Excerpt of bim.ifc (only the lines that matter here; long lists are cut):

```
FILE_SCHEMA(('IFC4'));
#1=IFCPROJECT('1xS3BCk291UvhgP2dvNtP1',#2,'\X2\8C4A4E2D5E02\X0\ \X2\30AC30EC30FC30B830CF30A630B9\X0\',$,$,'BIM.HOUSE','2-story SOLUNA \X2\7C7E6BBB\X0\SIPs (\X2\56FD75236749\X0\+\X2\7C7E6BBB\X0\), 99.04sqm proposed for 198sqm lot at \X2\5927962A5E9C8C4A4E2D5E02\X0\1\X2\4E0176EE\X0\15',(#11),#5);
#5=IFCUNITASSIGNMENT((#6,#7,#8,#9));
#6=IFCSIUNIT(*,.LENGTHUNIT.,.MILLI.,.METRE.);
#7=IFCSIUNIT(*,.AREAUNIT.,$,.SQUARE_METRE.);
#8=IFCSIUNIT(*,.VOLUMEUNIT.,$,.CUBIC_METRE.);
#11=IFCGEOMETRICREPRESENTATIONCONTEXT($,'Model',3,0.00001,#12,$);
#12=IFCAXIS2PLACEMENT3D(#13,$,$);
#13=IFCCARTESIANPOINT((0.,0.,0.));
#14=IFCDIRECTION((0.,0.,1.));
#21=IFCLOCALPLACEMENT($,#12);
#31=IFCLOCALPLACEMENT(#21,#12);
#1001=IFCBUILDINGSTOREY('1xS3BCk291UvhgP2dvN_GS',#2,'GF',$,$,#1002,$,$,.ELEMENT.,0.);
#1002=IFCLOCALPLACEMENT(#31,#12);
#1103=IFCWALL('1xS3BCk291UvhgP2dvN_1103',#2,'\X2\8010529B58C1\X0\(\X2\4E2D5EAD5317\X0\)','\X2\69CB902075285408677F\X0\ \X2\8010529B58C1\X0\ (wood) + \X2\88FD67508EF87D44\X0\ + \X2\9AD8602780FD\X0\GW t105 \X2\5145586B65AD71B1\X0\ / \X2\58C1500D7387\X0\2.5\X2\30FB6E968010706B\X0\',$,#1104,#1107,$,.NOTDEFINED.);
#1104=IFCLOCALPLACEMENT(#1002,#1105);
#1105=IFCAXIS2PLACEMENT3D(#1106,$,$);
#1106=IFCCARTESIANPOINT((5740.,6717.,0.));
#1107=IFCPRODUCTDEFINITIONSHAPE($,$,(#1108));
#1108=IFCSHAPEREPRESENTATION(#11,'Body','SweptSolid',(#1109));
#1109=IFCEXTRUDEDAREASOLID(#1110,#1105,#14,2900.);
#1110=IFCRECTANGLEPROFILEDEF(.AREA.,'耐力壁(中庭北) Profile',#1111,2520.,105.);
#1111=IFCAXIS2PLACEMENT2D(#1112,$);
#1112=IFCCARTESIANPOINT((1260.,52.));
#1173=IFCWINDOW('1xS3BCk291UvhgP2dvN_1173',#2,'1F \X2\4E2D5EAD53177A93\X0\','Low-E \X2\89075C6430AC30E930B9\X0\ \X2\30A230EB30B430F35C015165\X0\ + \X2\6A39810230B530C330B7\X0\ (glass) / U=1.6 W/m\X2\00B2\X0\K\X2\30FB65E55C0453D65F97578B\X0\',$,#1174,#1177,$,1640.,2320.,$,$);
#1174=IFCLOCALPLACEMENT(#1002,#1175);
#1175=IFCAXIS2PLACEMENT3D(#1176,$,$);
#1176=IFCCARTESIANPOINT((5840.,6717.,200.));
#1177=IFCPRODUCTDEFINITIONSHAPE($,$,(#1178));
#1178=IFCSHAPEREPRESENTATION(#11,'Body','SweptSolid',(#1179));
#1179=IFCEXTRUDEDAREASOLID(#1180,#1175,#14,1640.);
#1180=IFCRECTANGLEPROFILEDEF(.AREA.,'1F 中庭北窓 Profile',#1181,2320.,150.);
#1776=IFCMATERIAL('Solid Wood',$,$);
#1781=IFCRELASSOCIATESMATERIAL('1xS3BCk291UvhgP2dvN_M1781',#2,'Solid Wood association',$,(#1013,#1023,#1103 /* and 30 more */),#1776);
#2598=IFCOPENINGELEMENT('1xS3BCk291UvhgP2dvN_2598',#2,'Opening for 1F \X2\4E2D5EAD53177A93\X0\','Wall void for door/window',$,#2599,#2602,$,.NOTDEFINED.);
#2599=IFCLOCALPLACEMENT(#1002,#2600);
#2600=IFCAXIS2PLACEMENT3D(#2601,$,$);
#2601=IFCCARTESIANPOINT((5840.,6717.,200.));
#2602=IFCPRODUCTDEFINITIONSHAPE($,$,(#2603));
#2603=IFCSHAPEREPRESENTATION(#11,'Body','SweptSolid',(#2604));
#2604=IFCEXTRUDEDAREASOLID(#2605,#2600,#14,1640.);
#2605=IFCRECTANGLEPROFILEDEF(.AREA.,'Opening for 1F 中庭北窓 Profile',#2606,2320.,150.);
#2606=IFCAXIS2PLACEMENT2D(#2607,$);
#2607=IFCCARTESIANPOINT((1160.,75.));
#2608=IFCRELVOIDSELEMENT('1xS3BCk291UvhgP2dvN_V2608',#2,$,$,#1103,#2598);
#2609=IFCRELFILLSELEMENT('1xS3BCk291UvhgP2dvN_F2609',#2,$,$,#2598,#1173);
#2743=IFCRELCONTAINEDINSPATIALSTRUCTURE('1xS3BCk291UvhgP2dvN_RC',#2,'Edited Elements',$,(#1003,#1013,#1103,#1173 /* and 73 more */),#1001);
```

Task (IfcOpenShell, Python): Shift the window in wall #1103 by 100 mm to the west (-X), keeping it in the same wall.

```python
import ifcopenshell
import ifcopenshell.api.geometry
import ifcopenshell.util.placement

model = ifcopenshell.open("bim.ifc")

window = model.by_id(1173)
opening = window.FillsVoids[0].RelatingOpeningElement
wall = opening.VoidsElements[0].RelatingBuildingElement

wall_matrix = ifcopenshell.util.placement.get_local_placement(wall.ObjectPlacement)
shift = wall_matrix[:3, 0] * -100.0
before = ifcopenshell.util.placement.get_local_placement(window.ObjectPlacement)[:3, 3].copy()

# The window is not placed relative to its opening, so move both.
for product in (opening, window):
    matrix = ifcopenshell.util.placement.get_local_placement(product.ObjectPlacement)
    matrix[:3, 3] += shift
    ifcopenshell.api.geometry.edit_object_placement(model, product=product, matrix=matrix, is_si=False)

after = ifcopenshell.util.placement.get_local_placement(window.ObjectPlacement)[:3, 3]
print("window moved by", (after - before).round(3) + 0.0)

model.write("bim_updated.ifc")
```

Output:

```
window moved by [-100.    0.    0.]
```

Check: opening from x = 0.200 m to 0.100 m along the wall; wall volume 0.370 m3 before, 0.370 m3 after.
